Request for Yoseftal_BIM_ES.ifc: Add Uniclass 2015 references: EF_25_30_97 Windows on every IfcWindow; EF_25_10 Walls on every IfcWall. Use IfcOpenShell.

First a look at what the model holds.

```python
import ifcopenshell

model = ifcopenshell.open("Yoseftal_BIM_ES.ifc")
print(model.schema)
print("classifications:", [c.Name for c in model.by_type("IfcClassification")])
for ifc_class in ("IfcDoor", "IfcRoof", "IfcStair", "IfcWall", "IfcWindow"):
    print(ifc_class, len(model.by_type(ifc_class)))
```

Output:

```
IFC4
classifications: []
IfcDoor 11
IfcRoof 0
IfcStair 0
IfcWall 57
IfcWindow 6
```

```python
import ifcopenshell
import ifcopenshell.api.classification

model = ifcopenshell.open("Yoseftal_BIM_ES.ifc")

system = ifcopenshell.api.classification.add_classification(model, classification="Uniclass 2015")

codes = {
    "IfcWindow": ("EF_25_30_97", "Windows"),
    "IfcWall": ("EF_25_10", "Walls"),
}
for ifc_class, (code, name) in codes.items():
    products = model.by_type(ifc_class)
    ifcopenshell.api.classification.add_reference(
        model, products=products, classification=system, identification=code, name=name
    )
    print(code, len(products))

model.write("Yoseftal_BIM_ES_rev.ifc")
```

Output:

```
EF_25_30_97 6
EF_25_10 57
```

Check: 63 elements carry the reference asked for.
